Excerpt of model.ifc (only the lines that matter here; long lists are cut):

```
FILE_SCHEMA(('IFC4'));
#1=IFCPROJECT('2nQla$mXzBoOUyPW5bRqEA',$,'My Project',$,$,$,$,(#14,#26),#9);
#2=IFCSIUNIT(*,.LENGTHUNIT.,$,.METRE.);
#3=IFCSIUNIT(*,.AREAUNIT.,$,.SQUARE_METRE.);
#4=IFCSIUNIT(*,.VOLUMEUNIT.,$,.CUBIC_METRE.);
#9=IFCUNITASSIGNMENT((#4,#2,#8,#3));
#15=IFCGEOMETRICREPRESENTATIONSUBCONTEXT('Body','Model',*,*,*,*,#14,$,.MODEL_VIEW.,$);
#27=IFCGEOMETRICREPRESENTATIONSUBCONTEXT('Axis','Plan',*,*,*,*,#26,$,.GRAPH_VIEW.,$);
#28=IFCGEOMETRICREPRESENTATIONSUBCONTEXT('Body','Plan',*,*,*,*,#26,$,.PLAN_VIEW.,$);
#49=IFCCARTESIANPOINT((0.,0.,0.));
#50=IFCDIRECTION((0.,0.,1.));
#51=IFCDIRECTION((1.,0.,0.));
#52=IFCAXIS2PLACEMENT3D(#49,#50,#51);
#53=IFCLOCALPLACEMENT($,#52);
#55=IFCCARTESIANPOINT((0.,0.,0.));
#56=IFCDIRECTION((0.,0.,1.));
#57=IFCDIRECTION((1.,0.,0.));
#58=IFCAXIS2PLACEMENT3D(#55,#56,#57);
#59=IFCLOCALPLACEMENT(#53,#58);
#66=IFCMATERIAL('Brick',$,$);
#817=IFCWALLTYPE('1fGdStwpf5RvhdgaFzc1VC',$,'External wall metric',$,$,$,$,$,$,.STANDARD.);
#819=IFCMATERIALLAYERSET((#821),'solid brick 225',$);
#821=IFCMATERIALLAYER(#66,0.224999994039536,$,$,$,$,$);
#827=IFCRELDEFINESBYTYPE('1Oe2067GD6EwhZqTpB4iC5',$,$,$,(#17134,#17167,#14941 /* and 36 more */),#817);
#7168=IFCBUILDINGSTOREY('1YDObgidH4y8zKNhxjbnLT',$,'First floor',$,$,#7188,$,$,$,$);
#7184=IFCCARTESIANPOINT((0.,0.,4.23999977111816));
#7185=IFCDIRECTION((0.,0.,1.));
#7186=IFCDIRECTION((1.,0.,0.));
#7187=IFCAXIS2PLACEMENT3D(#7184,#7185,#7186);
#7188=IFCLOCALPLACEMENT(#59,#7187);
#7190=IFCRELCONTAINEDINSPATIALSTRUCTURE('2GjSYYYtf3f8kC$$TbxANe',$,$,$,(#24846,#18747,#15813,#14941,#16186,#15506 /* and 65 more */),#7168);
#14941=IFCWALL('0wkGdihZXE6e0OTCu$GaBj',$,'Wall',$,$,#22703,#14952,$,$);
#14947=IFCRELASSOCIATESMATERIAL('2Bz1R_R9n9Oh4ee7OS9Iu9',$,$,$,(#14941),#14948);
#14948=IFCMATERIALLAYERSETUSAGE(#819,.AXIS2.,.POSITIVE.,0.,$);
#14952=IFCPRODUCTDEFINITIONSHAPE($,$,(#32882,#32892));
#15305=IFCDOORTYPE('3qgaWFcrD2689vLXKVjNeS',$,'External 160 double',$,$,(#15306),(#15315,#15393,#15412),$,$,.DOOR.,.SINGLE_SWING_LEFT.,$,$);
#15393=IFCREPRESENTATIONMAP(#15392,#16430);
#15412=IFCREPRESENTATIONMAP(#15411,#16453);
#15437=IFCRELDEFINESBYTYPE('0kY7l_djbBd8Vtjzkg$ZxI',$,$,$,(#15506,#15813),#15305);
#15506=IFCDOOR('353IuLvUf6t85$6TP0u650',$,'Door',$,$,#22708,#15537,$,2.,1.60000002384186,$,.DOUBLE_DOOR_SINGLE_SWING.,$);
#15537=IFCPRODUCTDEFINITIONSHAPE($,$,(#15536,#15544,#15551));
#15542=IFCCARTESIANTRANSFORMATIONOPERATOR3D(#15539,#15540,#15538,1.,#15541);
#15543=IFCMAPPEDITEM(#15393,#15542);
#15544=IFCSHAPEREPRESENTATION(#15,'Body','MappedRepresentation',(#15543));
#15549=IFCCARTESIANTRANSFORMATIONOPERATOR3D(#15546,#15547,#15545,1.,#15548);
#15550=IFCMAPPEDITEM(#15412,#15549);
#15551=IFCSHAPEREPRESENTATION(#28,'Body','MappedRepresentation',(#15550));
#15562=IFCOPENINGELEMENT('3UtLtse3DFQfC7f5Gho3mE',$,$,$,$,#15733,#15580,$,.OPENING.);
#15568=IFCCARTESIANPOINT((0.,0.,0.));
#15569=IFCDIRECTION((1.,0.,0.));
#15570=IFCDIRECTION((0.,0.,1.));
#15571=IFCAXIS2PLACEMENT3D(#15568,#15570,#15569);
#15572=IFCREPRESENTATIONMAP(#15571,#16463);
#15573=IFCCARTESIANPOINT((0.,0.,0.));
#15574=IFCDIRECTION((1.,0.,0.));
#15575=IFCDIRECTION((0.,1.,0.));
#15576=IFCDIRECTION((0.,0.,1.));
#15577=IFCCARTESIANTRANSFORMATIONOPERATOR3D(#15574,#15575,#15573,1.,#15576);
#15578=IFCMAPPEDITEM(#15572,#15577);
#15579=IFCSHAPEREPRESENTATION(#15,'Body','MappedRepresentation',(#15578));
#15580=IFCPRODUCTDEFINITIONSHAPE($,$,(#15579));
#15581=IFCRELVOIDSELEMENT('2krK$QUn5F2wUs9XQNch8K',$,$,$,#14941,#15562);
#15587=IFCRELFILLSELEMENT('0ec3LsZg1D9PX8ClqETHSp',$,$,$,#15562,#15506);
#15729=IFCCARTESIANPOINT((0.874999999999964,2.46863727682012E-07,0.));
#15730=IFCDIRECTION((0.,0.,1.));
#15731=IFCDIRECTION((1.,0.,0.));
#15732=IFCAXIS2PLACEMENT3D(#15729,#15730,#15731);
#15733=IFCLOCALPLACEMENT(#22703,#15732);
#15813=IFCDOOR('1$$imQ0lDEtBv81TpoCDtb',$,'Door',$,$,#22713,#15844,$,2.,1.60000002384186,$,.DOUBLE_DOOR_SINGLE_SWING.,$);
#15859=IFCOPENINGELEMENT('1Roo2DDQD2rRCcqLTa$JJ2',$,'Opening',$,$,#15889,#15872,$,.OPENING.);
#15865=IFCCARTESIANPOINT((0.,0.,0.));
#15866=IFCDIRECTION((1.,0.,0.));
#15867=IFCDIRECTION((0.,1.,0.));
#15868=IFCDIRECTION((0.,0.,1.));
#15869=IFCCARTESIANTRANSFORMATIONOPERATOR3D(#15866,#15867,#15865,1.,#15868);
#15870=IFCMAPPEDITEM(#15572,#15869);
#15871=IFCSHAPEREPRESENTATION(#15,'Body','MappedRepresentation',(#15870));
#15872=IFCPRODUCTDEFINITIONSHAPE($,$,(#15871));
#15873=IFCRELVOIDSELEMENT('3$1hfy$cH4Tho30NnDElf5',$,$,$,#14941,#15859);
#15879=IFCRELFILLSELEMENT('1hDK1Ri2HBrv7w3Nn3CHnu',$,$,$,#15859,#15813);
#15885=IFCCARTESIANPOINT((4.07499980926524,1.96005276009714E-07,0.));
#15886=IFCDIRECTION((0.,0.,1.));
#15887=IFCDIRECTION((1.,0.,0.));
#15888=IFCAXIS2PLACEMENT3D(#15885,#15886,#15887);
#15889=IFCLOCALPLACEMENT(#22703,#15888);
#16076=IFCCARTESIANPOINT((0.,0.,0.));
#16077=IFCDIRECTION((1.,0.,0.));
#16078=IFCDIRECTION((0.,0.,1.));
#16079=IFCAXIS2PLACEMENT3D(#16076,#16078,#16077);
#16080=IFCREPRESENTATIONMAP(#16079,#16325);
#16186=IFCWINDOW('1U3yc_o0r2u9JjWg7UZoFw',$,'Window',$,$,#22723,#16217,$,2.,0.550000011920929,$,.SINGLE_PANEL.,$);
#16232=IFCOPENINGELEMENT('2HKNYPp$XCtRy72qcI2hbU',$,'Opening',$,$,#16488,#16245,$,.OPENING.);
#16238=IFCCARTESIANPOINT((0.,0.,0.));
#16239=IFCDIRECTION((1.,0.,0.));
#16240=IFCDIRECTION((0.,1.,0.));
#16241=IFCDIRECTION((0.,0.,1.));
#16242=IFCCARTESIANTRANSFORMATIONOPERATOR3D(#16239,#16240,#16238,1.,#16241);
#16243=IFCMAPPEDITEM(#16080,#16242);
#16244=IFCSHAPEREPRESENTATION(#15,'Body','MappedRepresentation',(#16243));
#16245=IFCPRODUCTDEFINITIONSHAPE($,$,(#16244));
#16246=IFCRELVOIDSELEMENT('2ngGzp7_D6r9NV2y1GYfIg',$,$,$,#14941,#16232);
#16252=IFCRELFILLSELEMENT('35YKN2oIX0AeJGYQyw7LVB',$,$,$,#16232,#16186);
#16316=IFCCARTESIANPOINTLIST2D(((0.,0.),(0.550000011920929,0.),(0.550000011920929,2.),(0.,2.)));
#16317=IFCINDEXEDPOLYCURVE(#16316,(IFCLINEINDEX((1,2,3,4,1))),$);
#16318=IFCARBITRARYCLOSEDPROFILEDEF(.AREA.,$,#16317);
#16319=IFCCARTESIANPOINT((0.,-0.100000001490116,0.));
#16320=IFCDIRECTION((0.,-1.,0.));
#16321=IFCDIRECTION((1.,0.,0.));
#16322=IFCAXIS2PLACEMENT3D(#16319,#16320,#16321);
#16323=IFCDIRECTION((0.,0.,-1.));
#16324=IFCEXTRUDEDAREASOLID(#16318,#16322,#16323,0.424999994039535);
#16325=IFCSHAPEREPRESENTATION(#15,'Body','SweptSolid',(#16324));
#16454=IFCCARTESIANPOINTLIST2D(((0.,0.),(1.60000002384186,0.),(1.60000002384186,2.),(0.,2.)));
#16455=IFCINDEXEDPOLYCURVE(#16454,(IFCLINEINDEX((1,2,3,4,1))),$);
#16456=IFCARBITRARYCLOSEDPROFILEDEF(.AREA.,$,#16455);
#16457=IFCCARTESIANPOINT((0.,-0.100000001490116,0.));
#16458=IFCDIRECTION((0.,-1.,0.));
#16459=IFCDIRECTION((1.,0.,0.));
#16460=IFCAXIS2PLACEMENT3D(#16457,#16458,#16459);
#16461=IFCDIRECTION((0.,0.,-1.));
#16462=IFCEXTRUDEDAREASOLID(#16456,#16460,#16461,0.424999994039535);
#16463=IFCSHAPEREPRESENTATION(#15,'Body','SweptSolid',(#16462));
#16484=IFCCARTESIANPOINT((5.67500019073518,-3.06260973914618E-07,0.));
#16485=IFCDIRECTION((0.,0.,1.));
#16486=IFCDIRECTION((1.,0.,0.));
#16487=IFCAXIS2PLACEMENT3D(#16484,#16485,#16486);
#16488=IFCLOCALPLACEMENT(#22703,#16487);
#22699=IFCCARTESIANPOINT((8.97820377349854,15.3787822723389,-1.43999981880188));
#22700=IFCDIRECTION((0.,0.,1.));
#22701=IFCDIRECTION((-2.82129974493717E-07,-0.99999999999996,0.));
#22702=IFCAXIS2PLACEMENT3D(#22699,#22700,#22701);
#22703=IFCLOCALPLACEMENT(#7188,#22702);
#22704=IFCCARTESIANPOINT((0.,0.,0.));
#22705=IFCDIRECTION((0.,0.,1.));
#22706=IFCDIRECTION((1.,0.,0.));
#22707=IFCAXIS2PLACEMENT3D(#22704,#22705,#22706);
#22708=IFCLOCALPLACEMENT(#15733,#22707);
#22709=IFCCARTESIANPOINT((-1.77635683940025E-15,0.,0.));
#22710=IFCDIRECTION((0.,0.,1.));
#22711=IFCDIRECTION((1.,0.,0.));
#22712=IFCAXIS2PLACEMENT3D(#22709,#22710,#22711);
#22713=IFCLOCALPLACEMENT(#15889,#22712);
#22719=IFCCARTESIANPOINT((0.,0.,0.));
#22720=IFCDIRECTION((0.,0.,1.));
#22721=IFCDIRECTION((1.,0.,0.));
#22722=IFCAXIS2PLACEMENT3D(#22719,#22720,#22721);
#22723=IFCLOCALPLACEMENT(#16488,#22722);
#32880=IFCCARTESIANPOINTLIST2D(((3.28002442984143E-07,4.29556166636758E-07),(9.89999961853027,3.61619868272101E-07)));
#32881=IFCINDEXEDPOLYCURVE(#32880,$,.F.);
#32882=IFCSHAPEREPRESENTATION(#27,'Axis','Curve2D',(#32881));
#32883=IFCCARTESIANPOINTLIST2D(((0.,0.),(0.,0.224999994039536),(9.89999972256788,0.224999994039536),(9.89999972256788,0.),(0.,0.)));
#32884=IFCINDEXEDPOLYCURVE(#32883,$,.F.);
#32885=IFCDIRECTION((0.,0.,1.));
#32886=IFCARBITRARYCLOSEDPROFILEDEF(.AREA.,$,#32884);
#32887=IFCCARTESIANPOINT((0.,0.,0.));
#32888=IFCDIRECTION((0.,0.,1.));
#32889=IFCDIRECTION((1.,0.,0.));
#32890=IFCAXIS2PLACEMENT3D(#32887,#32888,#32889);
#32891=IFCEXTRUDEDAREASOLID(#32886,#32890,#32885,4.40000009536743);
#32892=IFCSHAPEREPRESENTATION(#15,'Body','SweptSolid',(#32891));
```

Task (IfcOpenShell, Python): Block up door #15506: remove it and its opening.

```python
import ifcopenshell
import ifcopenshell.api.feature
import ifcopenshell.api.root
import ifcopenshell.geom
import ifcopenshell.util.shape

model = ifcopenshell.open("model.ifc")
settings = ifcopenshell.geom.settings()


def volume(element):
    """Net volume in cubic metres, openings subtracted."""
    shape = ifcopenshell.geom.create_shape(settings, element)
    return ifcopenshell.util.shape.get_volume(shape.geometry)


door = model.by_guid("353IuLvUf6t85$6TP0u650")
opening = door.FillsVoids[0].RelatingOpeningElement
wall = opening.VoidsElements[0].RelatingBuildingElement
before = volume(wall)

ifcopenshell.api.root.remove_product(model, product=door)
ifcopenshell.api.feature.remove_feature(model, feature=opening)

after = volume(wall)

print(f"wall volume {before:.3f} -> {after:.3f} m3")

model.write("model_updated.ifc")
```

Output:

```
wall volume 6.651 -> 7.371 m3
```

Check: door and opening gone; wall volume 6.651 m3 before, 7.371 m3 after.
